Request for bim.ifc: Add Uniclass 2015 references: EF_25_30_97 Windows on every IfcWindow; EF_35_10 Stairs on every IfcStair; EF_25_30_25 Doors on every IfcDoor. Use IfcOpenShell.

First a look at what the model holds.

```python
import ifcopenshell

model = ifcopenshell.open("bim.ifc")
print(model.schema)
print("classifications:", [c.Name for c in model.by_type("IfcClassification")])
for ifc_class in ("IfcDoor", "IfcRoof", "IfcStair", "IfcWall", "IfcWindow"):
    print(ifc_class, len(model.by_type(ifc_class)))
```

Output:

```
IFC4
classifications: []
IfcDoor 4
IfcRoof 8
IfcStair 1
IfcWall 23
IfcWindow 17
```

```python
import ifcopenshell
import ifcopenshell.api.classification

model = ifcopenshell.open("bim.ifc")

system = ifcopenshell.api.classification.add_classification(model, classification="Uniclass 2015")

codes = {
    "IfcWindow": ("EF_25_30_97", "Windows"),
    "IfcStair": ("EF_35_10", "Stairs"),
    "IfcDoor": ("EF_25_30_25", "Doors"),
}
for ifc_class, (code, name) in codes.items():
    products = model.by_type(ifc_class)
    ifcopenshell.api.classification.add_reference(
        model, products=products, classification=system, identification=code, name=name
    )
    print(code, len(products))

model.write("bim_v2.ifc")
```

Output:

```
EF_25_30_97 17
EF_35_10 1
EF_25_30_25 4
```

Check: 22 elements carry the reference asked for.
